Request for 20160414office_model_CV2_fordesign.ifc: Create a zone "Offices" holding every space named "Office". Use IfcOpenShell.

First a look at what the model holds.

```python
import ifcopenshell

model = ifcopenshell.open("20160414office_model_CV2_fordesign.ifc")
print(model.schema)
seen = {}
for space in model.by_type("IfcSpace"):
    seen[space.LongName] = seen.get(space.LongName, 0) + 1
for name, count in sorted(seen.items(), key=str):
    print(count, "x", name)
print("zones:", [z.Name for z in model.by_type("IfcZone")][:20])
```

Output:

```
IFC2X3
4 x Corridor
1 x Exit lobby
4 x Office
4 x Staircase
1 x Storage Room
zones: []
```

```python
import ifcopenshell
import ifcopenshell.api.group
import ifcopenshell.api.root

model = ifcopenshell.open("20160414office_model_CV2_fordesign.ifc")

names = {"Office"}
spaces = [s for s in model.by_type("IfcSpace") if s.LongName in names]

zone = ifcopenshell.api.root.create_entity(model, ifc_class="IfcZone", name="Offices")
ifcopenshell.api.group.assign_group(model, products=spaces, group=zone)
print(len(spaces), "spaces in", zone.Name)

model.write("20160414office_model_CV2_fordesign_updated.ifc")
```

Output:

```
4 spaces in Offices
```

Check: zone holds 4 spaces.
